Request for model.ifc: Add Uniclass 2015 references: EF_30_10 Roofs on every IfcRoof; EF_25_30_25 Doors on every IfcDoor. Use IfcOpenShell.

First a look at what the model holds.

```python
import ifcopenshell

model = ifcopenshell.open("model.ifc")
print(model.schema)
print("classifications:", [c.Name for c in model.by_type("IfcClassification")])
for ifc_class in ("IfcDoor", "IfcRoof", "IfcStair", "IfcWall", "IfcWindow"):
    print(ifc_class, len(model.by_type(ifc_class)))
```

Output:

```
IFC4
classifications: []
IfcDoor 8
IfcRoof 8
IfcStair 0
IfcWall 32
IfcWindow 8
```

```python
import ifcopenshell
import ifcopenshell.api.classification

model = ifcopenshell.open("model.ifc")

system = ifcopenshell.api.classification.add_classification(model, classification="Uniclass 2015")

codes = {
    "IfcRoof": ("EF_30_10", "Roofs"),
    "IfcDoor": ("EF_25_30_25", "Doors"),
}
for ifc_class, (code, name) in codes.items():
    products = model.by_type(ifc_class)
    ifcopenshell.api.classification.add_reference(
        model, products=products, classification=system, identification=code, name=name
    )
    print(code, len(products))

model.write("model_edited.ifc")
```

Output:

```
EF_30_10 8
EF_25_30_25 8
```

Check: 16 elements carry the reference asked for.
